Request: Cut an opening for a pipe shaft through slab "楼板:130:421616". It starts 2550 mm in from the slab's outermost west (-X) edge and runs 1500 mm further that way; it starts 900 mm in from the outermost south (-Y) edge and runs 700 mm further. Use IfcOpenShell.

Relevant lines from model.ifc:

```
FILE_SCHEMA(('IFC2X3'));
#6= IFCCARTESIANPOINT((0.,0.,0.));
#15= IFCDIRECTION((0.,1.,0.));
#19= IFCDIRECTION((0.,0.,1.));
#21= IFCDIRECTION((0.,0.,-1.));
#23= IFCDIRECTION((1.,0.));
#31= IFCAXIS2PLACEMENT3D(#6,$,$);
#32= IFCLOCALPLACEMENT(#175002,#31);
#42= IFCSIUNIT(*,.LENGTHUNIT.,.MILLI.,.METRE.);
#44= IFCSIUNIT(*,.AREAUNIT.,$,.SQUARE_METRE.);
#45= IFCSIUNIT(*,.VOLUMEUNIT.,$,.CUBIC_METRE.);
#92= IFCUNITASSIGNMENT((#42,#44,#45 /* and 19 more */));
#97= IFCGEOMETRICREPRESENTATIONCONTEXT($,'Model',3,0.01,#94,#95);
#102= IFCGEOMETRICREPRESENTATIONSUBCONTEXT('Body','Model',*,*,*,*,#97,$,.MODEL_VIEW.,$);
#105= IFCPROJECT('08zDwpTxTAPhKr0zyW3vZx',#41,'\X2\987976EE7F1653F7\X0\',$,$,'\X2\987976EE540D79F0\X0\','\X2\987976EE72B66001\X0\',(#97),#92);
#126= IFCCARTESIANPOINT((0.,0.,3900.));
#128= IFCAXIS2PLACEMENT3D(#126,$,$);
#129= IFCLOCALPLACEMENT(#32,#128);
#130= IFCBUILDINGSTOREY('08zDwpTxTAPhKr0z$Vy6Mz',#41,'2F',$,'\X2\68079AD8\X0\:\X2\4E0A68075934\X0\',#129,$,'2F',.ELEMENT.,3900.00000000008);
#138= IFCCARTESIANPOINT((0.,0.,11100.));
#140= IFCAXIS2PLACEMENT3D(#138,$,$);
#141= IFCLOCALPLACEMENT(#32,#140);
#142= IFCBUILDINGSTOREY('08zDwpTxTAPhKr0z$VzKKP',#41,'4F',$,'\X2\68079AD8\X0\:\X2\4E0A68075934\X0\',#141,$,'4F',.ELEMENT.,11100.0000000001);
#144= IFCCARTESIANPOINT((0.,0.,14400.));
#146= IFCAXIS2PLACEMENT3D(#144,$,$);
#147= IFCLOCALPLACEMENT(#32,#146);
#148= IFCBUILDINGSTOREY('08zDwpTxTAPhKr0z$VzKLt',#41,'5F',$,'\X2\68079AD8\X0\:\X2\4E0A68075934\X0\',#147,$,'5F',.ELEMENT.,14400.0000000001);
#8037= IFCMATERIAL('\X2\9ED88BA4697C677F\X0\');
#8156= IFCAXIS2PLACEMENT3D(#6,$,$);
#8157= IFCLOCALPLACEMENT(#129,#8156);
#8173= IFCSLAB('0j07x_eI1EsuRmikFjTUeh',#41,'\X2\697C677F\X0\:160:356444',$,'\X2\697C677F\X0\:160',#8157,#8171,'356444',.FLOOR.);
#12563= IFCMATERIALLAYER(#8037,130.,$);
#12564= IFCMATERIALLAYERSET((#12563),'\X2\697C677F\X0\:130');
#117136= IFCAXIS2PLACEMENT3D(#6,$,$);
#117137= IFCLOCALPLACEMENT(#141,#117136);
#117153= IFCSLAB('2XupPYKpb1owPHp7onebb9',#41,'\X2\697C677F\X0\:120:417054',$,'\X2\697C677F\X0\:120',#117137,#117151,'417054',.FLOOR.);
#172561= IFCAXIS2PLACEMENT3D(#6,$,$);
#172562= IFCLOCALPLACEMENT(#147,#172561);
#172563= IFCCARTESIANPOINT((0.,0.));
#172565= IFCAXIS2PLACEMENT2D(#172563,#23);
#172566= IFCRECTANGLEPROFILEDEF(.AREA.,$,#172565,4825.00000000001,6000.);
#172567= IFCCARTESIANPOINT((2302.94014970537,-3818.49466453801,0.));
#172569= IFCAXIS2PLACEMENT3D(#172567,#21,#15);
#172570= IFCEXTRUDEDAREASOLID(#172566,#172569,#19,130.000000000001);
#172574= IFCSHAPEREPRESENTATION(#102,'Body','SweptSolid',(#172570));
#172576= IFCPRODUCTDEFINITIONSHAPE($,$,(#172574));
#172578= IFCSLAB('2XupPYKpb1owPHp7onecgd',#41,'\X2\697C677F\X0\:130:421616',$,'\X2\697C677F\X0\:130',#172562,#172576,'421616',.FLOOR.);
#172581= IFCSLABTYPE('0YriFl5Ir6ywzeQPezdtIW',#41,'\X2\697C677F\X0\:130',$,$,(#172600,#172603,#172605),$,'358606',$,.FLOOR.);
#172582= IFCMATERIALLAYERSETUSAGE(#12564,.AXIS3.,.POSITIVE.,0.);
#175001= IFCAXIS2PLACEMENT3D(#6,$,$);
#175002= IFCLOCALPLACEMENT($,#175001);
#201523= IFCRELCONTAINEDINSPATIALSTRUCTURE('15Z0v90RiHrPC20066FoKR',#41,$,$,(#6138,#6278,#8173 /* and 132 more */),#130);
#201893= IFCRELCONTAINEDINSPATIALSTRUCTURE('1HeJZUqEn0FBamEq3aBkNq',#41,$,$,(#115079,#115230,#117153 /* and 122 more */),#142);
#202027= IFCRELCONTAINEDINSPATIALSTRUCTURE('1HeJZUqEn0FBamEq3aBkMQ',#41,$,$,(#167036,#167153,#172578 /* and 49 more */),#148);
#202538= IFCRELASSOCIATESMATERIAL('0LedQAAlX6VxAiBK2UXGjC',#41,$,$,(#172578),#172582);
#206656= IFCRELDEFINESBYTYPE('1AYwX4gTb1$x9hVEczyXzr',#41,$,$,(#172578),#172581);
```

```python
import numpy as np
import ifcopenshell
import ifcopenshell.api.feature
import ifcopenshell.api.geometry
import ifcopenshell.api.root
import ifcopenshell.geom
import ifcopenshell.util.placement
import ifcopenshell.util.representation
import ifcopenshell.util.shape
import ifcopenshell.util.unit

model = ifcopenshell.open("model.ifc")
unit_scale = ifcopenshell.util.unit.calculate_unit_scale(model)
settings = ifcopenshell.geom.settings()


def volume(element):
    """Net volume in cubic metres, openings subtracted."""
    shape = ifcopenshell.geom.create_shape(settings, element)
    return ifcopenshell.util.shape.get_volume(shape.geometry)


slab = model.by_guid("2XupPYKpb1owPHp7onecgd")
before = volume(slab)

# Extent in the slab's own axes, in metres. The edges named are its -X and -Y sides.
slab_shape = ifcopenshell.geom.create_shape(settings, slab)
vertices = ifcopenshell.util.shape.get_vertices(slab_shape.geometry)
x_min, y_min, bottom = vertices.min(axis=0)
top = vertices[:, 2].max()

opening = ifcopenshell.api.root.create_entity(model, ifc_class="IfcOpeningElement", name="Pipe shaft opening")
context = ifcopenshell.util.representation.get_context(model, "Model", "Body", "MODEL_VIEW")
width, depth = 1.5, 0.7
outline = [(0.0, 0.0), (width, 0.0), (width, depth), (0.0, depth), (0.0, 0.0)]
# Overshoot both faces by 50 mm so the cut is clean.
shape = ifcopenshell.api.geometry.add_slab_representation(
    model, context=context, depth=top - bottom + 0.1, polyline=outline
)
ifcopenshell.api.geometry.assign_representation(model, product=opening, representation=shape)

matrix = ifcopenshell.util.placement.get_local_placement(slab.ObjectPlacement)
matrix[:, 3] = matrix @ np.append(np.array([x_min + 2.55, y_min + 0.9, bottom - 0.05]) / unit_scale, 1.0)
ifcopenshell.api.geometry.edit_object_placement(model, product=opening, matrix=matrix, is_si=False)
ifcopenshell.api.feature.add_feature(model, feature=opening, element=slab)

after = volume(slab)

print(f"slab volume {before:.3f} -> {after:.3f} m3")

model.write("model_v2.ifc")
```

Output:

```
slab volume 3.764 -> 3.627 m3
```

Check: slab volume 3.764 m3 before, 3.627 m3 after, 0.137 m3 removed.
